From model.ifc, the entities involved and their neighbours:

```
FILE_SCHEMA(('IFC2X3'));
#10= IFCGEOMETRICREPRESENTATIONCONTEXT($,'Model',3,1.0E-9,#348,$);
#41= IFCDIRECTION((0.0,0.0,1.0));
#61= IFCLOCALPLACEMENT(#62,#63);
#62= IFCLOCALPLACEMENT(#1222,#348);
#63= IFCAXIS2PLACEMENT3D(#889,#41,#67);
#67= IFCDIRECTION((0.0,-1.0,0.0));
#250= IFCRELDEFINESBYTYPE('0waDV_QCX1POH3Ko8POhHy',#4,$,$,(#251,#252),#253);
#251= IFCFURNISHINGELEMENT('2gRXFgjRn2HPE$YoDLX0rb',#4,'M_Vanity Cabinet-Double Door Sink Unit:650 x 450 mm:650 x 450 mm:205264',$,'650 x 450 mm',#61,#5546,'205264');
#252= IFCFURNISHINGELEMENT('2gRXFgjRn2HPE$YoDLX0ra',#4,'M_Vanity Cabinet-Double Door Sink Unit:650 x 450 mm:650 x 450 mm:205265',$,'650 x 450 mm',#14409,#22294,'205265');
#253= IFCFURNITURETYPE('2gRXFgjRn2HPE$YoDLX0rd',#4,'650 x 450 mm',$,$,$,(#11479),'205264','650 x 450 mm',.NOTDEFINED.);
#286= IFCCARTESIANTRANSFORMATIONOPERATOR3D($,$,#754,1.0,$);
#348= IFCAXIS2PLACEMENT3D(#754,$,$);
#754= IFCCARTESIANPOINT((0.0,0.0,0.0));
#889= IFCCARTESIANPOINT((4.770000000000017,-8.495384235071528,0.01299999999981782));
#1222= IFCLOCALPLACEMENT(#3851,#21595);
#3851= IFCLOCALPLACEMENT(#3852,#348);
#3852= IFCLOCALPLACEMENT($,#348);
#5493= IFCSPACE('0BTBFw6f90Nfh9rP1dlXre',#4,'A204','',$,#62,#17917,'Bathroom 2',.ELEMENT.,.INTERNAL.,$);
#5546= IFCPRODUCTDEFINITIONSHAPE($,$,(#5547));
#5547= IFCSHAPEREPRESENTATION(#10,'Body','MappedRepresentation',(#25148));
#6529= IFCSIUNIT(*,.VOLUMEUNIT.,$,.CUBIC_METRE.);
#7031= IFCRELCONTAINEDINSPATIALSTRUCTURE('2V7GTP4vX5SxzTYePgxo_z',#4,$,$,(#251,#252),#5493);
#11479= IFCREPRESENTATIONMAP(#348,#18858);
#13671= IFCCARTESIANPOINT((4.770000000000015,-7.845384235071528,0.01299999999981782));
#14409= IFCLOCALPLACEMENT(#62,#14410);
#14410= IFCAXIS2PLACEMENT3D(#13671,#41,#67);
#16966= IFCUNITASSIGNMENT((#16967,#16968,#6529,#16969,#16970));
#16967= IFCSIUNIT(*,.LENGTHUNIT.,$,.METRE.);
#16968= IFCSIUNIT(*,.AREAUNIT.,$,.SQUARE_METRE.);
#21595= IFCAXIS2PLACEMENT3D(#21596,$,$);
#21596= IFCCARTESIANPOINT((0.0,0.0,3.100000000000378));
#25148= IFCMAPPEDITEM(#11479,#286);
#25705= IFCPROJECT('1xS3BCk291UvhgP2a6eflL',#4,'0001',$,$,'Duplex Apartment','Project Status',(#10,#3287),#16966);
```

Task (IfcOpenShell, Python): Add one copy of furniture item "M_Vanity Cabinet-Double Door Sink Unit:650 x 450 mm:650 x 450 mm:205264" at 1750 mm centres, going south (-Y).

```python
import numpy as np
import ifcopenshell
import ifcopenshell.api.geometry
import ifcopenshell.api.root
import ifcopenshell.util.element
import ifcopenshell.util.placement
import ifcopenshell.util.unit

model = ifcopenshell.open("model.ifc")
unit_scale = ifcopenshell.util.unit.calculate_unit_scale(model)


def reuse_history(source, copy):
    """copy_class also copies each property set's owner history, people and application; keep the originals."""
    for rel in copy.IsDefinedBy:
        if rel.is_a("IfcRelDefinesByProperties") and (history := rel.RelatingPropertyDefinition.OwnerHistory):
            rel.RelatingPropertyDefinition.OwnerHistory = source.OwnerHistory
            ifcopenshell.util.element.remove_deep2(model, history)


source = model.by_id(251)
base = ifcopenshell.util.placement.get_local_placement(source.ObjectPlacement)
step = np.array([0.0, -1.0, 0.0]) * 1.75 / unit_scale

for i in range(1, 2):
    copy = ifcopenshell.api.root.copy_class(model, product=source)
    copy.Representation = ifcopenshell.util.element.copy_deep(
        model, source.Representation, exclude=["IfcGeometricRepresentationContext", "IfcRepresentationMap"]
    )
    copy.Name = "M_Vanity Cabinet-Double Door Sink Unit:650 x 450 mm:650 x 450 mm"
    copy.Tag = None
    reuse_history(source, copy)
    matrix = base.copy()
    matrix[:3, 3] += i * step
    print("added at", matrix[:3, 3].round(3) + 0.0)
    ifcopenshell.api.geometry.edit_object_placement(model, product=copy, matrix=matrix, is_si=False)

model.write("model_v2.ifc")
```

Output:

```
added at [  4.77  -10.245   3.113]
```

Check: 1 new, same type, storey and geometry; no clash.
